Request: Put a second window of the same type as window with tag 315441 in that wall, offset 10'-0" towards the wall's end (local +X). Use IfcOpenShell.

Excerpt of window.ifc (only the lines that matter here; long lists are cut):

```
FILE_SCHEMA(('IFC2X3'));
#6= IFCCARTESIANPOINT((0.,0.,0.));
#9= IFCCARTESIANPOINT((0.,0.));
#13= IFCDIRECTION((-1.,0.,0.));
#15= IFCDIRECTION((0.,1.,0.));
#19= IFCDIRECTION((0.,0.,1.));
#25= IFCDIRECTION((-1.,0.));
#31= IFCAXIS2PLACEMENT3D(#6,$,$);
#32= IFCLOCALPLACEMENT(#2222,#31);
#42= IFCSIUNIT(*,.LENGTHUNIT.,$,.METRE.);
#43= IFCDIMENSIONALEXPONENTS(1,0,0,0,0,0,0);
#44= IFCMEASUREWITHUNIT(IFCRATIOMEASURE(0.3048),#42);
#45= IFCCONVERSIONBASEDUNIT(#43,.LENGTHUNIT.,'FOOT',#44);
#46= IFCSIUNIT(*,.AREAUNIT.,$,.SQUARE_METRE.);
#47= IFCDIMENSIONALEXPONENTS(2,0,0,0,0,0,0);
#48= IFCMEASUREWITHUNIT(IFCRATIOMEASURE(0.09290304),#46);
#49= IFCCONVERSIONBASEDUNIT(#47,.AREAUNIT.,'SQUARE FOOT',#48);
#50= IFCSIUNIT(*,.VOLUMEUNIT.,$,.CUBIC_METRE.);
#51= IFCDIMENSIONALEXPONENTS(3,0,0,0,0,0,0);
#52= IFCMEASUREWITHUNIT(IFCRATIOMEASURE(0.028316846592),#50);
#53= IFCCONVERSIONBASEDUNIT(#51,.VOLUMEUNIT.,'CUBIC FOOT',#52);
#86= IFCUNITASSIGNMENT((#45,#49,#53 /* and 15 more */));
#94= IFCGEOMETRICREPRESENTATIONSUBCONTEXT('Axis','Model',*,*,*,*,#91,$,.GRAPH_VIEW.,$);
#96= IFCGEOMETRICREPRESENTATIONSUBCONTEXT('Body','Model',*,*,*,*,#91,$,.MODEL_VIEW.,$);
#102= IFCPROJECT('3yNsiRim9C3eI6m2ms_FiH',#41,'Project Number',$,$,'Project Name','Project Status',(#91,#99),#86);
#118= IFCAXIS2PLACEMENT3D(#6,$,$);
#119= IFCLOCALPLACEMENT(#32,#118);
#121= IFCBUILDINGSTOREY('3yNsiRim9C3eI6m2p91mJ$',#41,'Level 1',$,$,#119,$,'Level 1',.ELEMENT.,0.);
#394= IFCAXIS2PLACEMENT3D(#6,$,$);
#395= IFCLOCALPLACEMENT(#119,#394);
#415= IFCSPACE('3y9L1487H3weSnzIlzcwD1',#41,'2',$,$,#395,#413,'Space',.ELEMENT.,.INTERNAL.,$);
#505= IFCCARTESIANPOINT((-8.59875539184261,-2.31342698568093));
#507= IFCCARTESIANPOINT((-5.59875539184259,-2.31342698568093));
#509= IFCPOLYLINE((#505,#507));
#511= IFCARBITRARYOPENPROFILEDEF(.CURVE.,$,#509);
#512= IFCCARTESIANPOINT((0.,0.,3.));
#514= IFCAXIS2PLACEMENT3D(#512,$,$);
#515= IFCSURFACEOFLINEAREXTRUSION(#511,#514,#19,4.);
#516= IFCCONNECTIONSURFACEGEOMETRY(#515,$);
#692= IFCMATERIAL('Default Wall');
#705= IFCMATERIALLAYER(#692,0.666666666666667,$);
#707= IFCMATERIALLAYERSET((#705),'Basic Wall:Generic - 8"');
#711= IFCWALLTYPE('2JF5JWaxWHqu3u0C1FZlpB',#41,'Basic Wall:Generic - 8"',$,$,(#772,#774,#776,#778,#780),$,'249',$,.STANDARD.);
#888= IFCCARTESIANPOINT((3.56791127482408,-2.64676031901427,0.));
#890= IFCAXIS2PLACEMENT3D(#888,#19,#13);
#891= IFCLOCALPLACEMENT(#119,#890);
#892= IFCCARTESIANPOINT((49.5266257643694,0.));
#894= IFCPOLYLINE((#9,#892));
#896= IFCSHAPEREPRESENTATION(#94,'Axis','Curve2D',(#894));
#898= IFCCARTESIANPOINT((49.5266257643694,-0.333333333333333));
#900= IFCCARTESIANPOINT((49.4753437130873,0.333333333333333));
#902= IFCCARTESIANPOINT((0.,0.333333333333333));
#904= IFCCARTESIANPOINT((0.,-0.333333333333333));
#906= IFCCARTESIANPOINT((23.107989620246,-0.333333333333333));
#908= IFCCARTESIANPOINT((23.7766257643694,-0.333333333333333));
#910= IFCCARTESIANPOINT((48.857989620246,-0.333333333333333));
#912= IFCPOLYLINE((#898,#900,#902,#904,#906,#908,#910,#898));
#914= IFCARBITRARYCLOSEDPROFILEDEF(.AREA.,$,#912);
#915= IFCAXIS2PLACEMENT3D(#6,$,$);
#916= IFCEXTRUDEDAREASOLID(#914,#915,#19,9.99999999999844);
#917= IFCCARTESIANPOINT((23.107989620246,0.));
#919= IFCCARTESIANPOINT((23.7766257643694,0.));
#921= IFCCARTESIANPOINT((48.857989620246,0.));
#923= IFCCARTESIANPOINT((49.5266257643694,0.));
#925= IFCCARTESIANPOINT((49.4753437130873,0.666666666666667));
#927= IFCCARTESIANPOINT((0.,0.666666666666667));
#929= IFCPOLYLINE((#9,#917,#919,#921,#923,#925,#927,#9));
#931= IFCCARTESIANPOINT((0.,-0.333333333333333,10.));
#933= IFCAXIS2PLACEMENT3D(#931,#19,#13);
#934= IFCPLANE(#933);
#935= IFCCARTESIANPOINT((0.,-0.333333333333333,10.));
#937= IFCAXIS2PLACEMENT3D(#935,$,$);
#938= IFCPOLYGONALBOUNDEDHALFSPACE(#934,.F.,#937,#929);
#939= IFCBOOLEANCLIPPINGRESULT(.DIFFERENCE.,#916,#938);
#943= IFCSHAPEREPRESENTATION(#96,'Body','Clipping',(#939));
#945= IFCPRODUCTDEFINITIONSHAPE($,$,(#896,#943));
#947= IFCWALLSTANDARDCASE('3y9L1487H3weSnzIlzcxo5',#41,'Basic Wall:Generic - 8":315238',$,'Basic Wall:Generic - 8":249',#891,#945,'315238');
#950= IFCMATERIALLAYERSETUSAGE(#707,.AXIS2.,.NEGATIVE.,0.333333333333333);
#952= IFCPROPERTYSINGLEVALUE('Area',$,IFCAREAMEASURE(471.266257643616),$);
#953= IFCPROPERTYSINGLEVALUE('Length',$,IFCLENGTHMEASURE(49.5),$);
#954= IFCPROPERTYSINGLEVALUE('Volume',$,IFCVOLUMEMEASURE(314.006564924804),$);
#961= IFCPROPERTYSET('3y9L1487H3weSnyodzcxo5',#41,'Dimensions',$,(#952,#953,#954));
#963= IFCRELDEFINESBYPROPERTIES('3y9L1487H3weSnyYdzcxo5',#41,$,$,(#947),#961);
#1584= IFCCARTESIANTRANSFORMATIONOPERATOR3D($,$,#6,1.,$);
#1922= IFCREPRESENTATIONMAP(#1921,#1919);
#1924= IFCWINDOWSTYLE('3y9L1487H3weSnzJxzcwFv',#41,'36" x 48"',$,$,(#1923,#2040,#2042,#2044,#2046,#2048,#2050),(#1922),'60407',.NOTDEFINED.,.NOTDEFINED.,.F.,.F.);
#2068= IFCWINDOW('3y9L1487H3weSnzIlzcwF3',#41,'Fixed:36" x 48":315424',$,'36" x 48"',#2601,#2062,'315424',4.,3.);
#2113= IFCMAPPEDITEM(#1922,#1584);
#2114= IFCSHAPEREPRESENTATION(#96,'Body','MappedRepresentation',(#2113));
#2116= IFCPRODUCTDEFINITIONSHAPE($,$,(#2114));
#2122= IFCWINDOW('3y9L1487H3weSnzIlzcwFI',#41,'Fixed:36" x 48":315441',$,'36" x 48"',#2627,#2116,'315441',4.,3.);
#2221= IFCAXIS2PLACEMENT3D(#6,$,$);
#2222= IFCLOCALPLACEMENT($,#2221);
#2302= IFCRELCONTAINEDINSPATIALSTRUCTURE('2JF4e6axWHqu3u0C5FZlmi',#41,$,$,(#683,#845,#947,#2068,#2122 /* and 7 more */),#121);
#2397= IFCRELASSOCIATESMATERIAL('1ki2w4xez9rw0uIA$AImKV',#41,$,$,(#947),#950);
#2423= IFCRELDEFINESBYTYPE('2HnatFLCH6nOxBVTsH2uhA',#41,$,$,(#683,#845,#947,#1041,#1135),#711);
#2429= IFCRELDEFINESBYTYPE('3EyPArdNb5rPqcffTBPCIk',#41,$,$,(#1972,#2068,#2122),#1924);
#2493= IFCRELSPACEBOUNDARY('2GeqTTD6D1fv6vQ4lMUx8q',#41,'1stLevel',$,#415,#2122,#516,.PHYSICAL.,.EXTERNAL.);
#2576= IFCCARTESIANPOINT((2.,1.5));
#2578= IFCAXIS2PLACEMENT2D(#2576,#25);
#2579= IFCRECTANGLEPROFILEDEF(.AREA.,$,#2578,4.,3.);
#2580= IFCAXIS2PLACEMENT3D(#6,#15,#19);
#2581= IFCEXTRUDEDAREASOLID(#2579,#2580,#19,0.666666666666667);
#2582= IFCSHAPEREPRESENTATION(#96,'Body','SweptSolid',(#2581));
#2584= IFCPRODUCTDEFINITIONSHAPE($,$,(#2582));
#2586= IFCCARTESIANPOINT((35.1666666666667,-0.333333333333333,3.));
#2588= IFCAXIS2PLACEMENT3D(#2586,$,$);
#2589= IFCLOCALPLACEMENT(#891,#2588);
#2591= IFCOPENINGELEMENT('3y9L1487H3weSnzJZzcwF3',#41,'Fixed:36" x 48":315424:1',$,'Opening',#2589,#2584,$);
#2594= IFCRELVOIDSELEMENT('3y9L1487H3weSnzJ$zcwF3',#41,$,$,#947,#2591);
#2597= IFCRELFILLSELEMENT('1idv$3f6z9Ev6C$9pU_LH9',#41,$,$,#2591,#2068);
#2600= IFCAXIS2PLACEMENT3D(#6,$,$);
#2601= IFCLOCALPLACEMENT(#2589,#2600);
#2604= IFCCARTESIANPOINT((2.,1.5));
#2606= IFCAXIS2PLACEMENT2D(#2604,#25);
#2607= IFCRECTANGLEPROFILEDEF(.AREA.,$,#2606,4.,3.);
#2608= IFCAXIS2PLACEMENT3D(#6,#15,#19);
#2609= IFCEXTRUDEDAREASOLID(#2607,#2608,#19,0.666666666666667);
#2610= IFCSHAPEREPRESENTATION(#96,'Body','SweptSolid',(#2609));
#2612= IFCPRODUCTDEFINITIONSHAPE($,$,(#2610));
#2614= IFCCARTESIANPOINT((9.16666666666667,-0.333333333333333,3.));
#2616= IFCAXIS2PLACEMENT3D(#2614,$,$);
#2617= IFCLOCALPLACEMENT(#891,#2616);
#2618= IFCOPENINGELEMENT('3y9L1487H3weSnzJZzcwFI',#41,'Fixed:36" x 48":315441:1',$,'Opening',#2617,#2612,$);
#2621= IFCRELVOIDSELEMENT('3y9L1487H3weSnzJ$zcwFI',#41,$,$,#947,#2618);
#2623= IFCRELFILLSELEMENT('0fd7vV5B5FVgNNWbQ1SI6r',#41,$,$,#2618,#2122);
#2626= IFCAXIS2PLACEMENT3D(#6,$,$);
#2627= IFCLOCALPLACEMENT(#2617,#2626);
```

```python
import numpy as np
import ifcopenshell
import ifcopenshell.api.feature
import ifcopenshell.api.geometry
import ifcopenshell.api.pset
import ifcopenshell.api.root
import ifcopenshell.geom
import ifcopenshell.util.element
import ifcopenshell.util.placement
import ifcopenshell.util.shape
import ifcopenshell.util.unit

model = ifcopenshell.open("window.ifc")
unit_scale = ifcopenshell.util.unit.calculate_unit_scale(model)
area_scale = ifcopenshell.util.unit.calculate_unit_scale(model, "AREAUNIT")
volume_scale = ifcopenshell.util.unit.calculate_unit_scale(model, "VOLUMEUNIT")
settings = ifcopenshell.geom.settings()


def volume(element):
    """Net volume in cubic metres, openings subtracted."""
    shape = ifcopenshell.geom.create_shape(settings, element)
    return ifcopenshell.util.shape.get_volume(shape.geometry)


def reuse_history(source, copy):
    """copy_class also copies each property set's owner history, people and application; keep the originals."""
    for rel in copy.IsDefinedBy:
        if rel.is_a("IfcRelDefinesByProperties") and (history := rel.RelatingPropertyDefinition.OwnerHistory):
            rel.RelatingPropertyDefinition.OwnerHistory = source.OwnerHistory
            ifcopenshell.util.element.remove_deep2(model, history)


window = model.by_guid("3y9L1487H3weSnzIlzcwFI")
opening = window.FillsVoids[0].RelatingOpeningElement
wall = opening.VoidsElements[0].RelatingBuildingElement
before = volume(wall)
shift = ifcopenshell.util.placement.get_local_placement(wall.ObjectPlacement)[:3, 0] * 120 * 0.0254 / unit_scale

# copy_class copies the void relationship, type, container and properties, but no geometry.
new_opening = ifcopenshell.api.root.copy_class(model, product=opening)
new_opening.Representation = ifcopenshell.util.element.copy_deep(
    model, opening.Representation, exclude=["IfcGeometricRepresentationContext", "IfcRepresentationMap"]
)
new_opening.Name = 'Fixed:36" x 48"'
new_window = ifcopenshell.api.root.copy_class(model, product=window)
new_window.Representation = ifcopenshell.util.element.copy_deep(
    model, window.Representation, exclude=["IfcGeometricRepresentationContext", "IfcRepresentationMap"]
)
new_window.Name = 'Fixed:36" x 48"'
new_window.Tag = None
reuse_history(window, new_window)
fills = ifcopenshell.api.feature.add_filling(model, opening=new_opening, element=new_window)
fills.OwnerHistory = new_window.OwnerHistory  # required in IFC2X3

for old, new in ((opening, new_opening), (window, new_window)):
    matrix = ifcopenshell.util.placement.get_local_placement(old.ObjectPlacement)
    matrix[:3, 3] += shift
    ifcopenshell.api.geometry.edit_object_placement(model, product=new, matrix=matrix, is_si=False)

# The copied space boundaries still share their surfaces with the original.
for rel in new_window.ProvidesBoundaries:
    if rel.ConnectionGeometry:
        rel.ConnectionGeometry = ifcopenshell.util.element.copy_deep(model, rel.ConnectionGeometry)

# Space boundary surfaces are stored in each space's coordinates; move them too.
for rel in new_window.ProvidesBoundaries:
    if not rel.ConnectionGeometry:
        continue
    surface = rel.ConnectionGeometry.SurfaceOnRelatingElement
    space_matrix = ifcopenshell.util.placement.get_local_placement(rel.RelatingSpace.ObjectPlacement)
    point = np.array(surface.Position.Location.Coordinates) + space_matrix[:3, :3].T @ shift
    surface.Position = model.createIfcAxis2Placement3D(
        model.createIfcCartesianPoint(point.tolist()), surface.Position.Axis, surface.Position.RefDirection
    )

after = volume(wall)
thickness = 0.2032  # wall thickness in metres

# Update the wall's stored quantities.
pset = model.by_id(ifcopenshell.util.element.get_pset(wall, "Dimensions", should_inherit=False)["id"])
ifcopenshell.api.pset.edit_pset(model, pset=pset, properties={
    "Area": model.create_entity("IfcAreaMeasure", after / thickness / area_scale),
    "Volume": model.create_entity("IfcVolumeMeasure", after / volume_scale),
})

print(f"wall volume {before:.3f} -> {after:.3f} m3")

model.write("window_v2.ifc")
```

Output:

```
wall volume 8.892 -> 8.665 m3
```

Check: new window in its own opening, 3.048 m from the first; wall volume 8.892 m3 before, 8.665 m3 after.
